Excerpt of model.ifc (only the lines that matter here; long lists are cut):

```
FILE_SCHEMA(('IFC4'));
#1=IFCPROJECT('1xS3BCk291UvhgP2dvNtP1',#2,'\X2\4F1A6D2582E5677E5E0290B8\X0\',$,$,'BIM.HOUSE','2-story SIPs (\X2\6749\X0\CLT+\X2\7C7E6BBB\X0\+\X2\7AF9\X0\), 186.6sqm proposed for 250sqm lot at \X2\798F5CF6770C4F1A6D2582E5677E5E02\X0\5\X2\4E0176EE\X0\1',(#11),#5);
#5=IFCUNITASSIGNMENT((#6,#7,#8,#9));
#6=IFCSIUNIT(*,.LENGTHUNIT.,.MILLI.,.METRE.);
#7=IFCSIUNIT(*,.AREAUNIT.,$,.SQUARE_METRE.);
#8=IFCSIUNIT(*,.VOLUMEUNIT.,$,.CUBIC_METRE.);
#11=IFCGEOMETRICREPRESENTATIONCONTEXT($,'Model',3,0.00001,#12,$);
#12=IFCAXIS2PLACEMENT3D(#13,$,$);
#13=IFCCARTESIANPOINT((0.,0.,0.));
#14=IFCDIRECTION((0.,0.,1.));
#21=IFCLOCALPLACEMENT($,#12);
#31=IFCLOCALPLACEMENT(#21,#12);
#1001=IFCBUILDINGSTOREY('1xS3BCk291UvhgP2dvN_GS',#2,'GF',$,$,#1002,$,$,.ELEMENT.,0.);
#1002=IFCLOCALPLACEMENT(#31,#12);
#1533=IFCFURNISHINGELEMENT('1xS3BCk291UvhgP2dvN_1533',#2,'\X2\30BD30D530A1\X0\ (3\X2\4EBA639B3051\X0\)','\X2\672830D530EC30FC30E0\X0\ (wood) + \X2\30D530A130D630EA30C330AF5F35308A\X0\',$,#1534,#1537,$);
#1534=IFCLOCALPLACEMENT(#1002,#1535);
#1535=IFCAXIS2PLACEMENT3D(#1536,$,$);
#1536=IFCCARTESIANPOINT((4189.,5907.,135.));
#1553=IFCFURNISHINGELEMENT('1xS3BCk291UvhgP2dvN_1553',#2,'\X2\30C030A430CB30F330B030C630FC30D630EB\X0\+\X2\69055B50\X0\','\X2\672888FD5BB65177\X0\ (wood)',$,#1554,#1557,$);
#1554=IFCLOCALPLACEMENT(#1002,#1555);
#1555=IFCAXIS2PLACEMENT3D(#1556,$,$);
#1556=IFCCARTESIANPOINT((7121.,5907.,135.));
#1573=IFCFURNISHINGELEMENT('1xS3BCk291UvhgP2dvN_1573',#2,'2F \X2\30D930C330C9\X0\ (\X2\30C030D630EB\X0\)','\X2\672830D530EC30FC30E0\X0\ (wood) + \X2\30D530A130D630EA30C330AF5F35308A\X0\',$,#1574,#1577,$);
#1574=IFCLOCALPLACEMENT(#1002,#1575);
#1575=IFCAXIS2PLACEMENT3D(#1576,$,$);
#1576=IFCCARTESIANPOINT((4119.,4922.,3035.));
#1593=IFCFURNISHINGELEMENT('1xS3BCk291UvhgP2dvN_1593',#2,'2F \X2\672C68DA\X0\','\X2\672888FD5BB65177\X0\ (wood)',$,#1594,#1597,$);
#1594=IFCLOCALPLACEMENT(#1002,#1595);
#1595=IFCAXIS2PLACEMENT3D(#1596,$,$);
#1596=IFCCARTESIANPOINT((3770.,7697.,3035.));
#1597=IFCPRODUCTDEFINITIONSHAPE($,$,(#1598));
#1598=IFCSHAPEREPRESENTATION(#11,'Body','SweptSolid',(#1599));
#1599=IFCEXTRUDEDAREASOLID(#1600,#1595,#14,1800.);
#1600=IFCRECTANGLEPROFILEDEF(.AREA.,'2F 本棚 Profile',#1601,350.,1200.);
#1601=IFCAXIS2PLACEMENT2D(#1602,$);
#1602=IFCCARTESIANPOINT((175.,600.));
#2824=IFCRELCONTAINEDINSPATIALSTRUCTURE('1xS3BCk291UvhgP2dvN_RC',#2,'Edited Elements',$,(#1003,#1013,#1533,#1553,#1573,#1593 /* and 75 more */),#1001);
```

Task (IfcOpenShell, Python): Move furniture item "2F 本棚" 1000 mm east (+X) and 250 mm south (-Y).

```python
import ifcopenshell
import ifcopenshell.api.geometry
import ifcopenshell.util.placement

model = ifcopenshell.open("model.ifc")

item = model.by_guid("1xS3BCk291UvhgP2dvN_1593")
matrix = ifcopenshell.util.placement.get_local_placement(item.ObjectPlacement)
matrix[0, 3] += 1000.0
matrix[1, 3] -= 250.0
ifcopenshell.api.geometry.edit_object_placement(model, product=item, matrix=matrix, is_si=False)

print(ifcopenshell.util.placement.get_local_placement(item.ObjectPlacement).round(3) + 0.0)

model.write("model_edited.ifc")
```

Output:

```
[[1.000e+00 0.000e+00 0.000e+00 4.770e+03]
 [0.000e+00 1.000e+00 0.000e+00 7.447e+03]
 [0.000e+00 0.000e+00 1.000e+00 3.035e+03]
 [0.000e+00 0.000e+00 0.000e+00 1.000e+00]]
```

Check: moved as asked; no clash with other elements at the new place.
